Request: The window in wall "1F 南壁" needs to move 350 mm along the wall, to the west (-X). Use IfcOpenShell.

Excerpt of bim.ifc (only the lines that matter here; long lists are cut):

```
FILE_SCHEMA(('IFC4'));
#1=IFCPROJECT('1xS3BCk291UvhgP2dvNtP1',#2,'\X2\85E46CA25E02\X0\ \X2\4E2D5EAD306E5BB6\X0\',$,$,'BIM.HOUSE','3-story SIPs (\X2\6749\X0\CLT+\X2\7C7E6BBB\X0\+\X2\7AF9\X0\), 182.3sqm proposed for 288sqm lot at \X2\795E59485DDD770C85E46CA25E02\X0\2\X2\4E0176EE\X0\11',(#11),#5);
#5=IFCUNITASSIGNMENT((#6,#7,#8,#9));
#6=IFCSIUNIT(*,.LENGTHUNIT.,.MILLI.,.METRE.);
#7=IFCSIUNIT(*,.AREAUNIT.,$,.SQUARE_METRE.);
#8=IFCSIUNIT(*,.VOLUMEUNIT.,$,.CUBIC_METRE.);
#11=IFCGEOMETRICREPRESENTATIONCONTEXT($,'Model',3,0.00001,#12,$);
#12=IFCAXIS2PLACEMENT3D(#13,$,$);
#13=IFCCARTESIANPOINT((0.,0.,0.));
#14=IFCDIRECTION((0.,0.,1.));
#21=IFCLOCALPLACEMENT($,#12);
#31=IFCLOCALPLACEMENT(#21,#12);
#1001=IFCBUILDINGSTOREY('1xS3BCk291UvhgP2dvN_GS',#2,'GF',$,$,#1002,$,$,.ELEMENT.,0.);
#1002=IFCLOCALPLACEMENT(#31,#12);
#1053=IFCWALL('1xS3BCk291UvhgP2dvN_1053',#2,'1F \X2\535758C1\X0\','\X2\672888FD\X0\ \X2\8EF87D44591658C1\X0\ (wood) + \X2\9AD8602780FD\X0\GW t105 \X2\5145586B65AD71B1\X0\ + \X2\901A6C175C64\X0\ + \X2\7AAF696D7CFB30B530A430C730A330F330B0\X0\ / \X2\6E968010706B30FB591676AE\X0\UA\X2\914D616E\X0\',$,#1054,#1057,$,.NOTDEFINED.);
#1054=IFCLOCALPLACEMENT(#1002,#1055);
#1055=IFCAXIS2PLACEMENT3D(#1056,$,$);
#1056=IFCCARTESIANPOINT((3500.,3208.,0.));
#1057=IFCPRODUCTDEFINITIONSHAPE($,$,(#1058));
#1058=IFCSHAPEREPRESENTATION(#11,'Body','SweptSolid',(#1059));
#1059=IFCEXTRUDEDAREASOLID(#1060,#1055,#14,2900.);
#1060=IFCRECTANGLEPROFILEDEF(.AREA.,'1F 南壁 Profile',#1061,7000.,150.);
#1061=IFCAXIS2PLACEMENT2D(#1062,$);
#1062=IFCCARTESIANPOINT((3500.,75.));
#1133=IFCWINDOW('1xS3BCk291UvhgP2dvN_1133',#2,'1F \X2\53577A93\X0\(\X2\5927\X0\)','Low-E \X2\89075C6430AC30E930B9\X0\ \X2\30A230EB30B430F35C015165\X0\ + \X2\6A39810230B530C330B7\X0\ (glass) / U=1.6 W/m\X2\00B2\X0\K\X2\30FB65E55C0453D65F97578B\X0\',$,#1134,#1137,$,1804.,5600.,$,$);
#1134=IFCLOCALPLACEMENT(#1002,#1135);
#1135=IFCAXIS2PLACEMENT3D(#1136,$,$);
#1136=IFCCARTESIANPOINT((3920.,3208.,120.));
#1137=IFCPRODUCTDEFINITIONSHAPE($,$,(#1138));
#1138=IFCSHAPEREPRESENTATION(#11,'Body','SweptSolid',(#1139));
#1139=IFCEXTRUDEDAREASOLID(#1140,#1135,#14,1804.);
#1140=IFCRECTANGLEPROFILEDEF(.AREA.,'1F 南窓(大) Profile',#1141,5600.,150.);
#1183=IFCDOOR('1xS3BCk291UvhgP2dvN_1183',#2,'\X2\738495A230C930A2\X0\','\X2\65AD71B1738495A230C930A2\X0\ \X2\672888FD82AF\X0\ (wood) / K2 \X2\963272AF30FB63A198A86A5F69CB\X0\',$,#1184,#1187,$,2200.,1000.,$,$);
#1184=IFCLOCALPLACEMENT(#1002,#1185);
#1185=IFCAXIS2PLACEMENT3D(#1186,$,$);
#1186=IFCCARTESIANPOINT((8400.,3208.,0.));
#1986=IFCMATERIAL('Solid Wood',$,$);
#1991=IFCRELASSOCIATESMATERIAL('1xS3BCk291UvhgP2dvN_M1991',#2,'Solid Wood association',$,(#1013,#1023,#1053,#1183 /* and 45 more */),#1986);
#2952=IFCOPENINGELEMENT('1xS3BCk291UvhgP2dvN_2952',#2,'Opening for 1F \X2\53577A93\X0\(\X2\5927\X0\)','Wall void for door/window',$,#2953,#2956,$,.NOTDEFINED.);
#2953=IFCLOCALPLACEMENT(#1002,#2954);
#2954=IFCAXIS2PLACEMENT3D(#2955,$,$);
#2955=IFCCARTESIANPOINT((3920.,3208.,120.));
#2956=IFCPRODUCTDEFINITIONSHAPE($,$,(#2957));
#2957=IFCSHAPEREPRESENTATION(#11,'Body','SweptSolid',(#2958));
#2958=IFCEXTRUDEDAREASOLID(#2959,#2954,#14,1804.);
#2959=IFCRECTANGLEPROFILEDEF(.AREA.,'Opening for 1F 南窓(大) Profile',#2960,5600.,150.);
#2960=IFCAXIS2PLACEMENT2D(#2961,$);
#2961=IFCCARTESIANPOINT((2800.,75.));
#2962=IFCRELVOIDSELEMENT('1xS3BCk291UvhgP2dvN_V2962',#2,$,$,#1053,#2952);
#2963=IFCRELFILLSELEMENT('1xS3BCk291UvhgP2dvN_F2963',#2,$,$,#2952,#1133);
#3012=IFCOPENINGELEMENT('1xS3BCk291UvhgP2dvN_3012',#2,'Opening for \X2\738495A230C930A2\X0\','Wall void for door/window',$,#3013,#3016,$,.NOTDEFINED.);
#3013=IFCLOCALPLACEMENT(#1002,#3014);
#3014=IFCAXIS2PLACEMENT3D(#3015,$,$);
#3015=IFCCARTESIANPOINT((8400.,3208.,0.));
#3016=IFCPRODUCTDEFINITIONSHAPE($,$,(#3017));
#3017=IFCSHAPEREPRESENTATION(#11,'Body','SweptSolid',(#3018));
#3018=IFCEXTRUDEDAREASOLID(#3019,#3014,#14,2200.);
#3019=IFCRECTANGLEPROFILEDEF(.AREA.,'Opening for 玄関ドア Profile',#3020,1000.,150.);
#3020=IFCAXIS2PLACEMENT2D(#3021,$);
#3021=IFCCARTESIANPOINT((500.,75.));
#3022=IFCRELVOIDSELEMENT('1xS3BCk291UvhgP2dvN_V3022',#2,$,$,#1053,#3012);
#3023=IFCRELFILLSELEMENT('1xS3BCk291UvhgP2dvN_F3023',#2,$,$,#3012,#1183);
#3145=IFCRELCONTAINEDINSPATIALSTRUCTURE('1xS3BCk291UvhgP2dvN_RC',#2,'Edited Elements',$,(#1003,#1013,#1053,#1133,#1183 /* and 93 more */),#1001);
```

```python
import ifcopenshell
import ifcopenshell.api.geometry
import ifcopenshell.util.placement
import ifcopenshell.util.unit

model = ifcopenshell.open("bim.ifc")
unit_scale = ifcopenshell.util.unit.calculate_unit_scale(model)

window = model.by_guid("1xS3BCk291UvhgP2dvN_1133")
opening = window.FillsVoids[0].RelatingOpeningElement
wall = opening.VoidsElements[0].RelatingBuildingElement

wall_matrix = ifcopenshell.util.placement.get_local_placement(wall.ObjectPlacement)
shift = wall_matrix[:3, 0] * -0.35 / unit_scale
before = ifcopenshell.util.placement.get_local_placement(window.ObjectPlacement)[:3, 3].copy()

# The window is not placed relative to its opening, so move both.
for product in (opening, window):
    matrix = ifcopenshell.util.placement.get_local_placement(product.ObjectPlacement)
    matrix[:3, 3] += shift
    ifcopenshell.api.geometry.edit_object_placement(model, product=product, matrix=matrix, is_si=False)

after = ifcopenshell.util.placement.get_local_placement(window.ObjectPlacement)[:3, 3]
print("window moved by", (after - before).round(3) + 0.0)

model.write("bim_rev.ifc")
```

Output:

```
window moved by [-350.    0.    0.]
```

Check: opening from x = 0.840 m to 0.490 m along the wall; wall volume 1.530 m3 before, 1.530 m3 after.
